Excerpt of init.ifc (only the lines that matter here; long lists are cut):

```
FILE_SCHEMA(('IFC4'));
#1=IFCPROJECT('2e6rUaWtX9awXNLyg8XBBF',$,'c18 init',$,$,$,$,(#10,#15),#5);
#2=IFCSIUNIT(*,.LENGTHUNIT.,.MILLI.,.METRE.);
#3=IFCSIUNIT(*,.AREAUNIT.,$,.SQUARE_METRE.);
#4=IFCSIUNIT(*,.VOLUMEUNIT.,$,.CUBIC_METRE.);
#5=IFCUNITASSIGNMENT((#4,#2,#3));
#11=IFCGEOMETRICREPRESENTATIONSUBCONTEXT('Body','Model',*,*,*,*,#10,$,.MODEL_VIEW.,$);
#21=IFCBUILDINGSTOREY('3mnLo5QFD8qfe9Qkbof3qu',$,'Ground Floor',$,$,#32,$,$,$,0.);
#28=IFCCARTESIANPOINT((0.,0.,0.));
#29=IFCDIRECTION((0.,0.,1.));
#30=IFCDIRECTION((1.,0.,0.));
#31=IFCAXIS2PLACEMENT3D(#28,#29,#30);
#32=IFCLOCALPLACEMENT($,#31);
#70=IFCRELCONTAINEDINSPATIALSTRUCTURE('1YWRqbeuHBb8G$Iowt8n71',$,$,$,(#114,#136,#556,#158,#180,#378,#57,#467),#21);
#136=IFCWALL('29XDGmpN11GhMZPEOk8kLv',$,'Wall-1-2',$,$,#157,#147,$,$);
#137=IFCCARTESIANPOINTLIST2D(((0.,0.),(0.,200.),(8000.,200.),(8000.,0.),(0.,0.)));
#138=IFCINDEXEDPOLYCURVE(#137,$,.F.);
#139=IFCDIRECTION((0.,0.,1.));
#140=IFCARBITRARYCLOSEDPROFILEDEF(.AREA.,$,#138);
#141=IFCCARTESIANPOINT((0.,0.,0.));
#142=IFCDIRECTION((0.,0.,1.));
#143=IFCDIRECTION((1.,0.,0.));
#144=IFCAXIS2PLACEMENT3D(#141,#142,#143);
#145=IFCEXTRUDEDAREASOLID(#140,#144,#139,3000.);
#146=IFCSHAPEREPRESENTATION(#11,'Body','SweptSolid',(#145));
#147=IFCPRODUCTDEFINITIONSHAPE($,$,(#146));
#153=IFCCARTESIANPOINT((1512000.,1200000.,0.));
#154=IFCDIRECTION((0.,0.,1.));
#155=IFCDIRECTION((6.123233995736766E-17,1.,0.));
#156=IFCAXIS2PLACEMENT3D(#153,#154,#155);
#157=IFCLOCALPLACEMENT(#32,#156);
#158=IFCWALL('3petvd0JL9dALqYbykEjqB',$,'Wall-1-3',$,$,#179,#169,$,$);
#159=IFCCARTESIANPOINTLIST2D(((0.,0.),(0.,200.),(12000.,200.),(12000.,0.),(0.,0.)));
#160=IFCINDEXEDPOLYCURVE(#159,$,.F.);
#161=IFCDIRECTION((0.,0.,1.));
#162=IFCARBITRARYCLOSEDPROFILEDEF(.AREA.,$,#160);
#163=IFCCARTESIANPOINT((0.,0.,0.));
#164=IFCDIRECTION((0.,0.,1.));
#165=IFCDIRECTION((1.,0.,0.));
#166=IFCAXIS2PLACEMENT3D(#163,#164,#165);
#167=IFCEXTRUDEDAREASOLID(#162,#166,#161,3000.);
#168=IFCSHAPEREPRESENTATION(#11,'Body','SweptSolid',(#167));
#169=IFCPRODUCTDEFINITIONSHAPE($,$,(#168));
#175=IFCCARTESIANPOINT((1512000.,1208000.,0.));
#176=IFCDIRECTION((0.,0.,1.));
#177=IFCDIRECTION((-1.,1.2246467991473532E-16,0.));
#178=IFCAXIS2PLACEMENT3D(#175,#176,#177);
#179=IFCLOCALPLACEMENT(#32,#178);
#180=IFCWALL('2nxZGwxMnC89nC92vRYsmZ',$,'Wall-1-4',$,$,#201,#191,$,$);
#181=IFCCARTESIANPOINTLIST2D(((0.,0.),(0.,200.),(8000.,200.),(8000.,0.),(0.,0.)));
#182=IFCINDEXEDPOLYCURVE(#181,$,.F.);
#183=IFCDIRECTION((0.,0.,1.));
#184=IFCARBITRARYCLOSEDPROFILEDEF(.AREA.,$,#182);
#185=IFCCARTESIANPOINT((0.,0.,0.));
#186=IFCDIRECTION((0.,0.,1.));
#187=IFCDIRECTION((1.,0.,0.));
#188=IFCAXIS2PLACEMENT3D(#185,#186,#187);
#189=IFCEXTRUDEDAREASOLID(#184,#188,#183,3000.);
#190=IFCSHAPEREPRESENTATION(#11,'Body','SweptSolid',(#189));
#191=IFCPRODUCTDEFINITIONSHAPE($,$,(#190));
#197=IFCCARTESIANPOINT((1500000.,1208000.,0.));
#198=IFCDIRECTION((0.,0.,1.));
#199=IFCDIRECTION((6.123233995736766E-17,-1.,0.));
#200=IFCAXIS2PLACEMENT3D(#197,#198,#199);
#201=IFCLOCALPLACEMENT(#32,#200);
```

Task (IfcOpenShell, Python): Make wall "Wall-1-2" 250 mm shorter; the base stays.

```python
import ifcopenshell
import ifcopenshell.geom
import ifcopenshell.util.representation
import ifcopenshell.util.shape
import ifcopenshell.util.unit

model = ifcopenshell.open("init.ifc")
unit_scale = ifcopenshell.util.unit.calculate_unit_scale(model)
settings = ifcopenshell.geom.settings()


def volume(element):
    """Net volume in cubic metres, openings subtracted."""
    shape = ifcopenshell.geom.create_shape(settings, element)
    return ifcopenshell.util.shape.get_volume(shape.geometry)


wall = model.by_guid("29XDGmpN11GhMZPEOk8kLv")
before = volume(wall)

body = ifcopenshell.util.representation.get_representation(wall, "Model", "Body")
solid = body.Items[0]
old_height = solid.Depth
solid.Depth -= 0.25 / unit_scale
after = volume(wall)

print(f"height {old_height:g} -> {solid.Depth:g}, volume {before:.3f} -> {after:.3f} m3")

model.write("init_v2.ifc")
```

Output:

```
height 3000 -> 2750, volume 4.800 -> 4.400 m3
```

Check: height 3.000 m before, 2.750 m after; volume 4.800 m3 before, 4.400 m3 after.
